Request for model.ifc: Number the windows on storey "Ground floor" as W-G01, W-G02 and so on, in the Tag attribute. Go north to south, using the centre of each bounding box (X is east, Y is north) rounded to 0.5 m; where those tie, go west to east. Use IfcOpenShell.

First a look at what the model holds.

```python
import ifcopenshell
import ifcopenshell.util.element
import ifcopenshell.util.placement

model = ifcopenshell.open("model.ifc")
print(model.schema)
storey = next(s for s in model.by_type("IfcBuildingStorey") if s.Name == "Ground floor")
windows = [e for e in ifcopenshell.util.element.get_decomposition(storey) if e.is_a("IfcWindow")]
for e in sorted(windows, key=lambda e: e.id()):
    origin = ifcopenshell.util.placement.get_local_placement(e.ObjectPlacement)[:3, 3]
    print(e.id(), e.Tag, e.Name, origin.round(2) + 0.0, sep=" | ")
```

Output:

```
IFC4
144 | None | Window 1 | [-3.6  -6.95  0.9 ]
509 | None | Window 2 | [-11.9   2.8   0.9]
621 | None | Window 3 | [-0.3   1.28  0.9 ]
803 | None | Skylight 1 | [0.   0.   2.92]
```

```python
import ifcopenshell
import ifcopenshell.geom
import ifcopenshell.util.element
import ifcopenshell.util.shape

model = ifcopenshell.open("model.ifc")
settings = ifcopenshell.geom.settings()
settings.set("use-world-coords", True)


def centre(element):
    shape = ifcopenshell.geom.create_shape(settings, element)
    return ifcopenshell.util.shape.get_bbox_centroid(shape.geometry)


storey = next(s for s in model.by_type("IfcBuildingStorey") if s.Name == "Ground floor")
windows = [e for e in ifcopenshell.util.element.get_decomposition(storey) if e.is_a("IfcWindow")]

# Insertion points can sit at a corner or the storey origin, so sort by the geometry (in metres).
centres = {e: centre(e) for e in windows}
windows.sort(key=lambda e: (-round(centres[e][1] / 0.5), centres[e][0]))

for i, e in enumerate(windows, start=1):
    number = f"W-G{i:02d}"
    e.Tag = number
    print(e.id(), number)

model.write("model_updated.ifc")
```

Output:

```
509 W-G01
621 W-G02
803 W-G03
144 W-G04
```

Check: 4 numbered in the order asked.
